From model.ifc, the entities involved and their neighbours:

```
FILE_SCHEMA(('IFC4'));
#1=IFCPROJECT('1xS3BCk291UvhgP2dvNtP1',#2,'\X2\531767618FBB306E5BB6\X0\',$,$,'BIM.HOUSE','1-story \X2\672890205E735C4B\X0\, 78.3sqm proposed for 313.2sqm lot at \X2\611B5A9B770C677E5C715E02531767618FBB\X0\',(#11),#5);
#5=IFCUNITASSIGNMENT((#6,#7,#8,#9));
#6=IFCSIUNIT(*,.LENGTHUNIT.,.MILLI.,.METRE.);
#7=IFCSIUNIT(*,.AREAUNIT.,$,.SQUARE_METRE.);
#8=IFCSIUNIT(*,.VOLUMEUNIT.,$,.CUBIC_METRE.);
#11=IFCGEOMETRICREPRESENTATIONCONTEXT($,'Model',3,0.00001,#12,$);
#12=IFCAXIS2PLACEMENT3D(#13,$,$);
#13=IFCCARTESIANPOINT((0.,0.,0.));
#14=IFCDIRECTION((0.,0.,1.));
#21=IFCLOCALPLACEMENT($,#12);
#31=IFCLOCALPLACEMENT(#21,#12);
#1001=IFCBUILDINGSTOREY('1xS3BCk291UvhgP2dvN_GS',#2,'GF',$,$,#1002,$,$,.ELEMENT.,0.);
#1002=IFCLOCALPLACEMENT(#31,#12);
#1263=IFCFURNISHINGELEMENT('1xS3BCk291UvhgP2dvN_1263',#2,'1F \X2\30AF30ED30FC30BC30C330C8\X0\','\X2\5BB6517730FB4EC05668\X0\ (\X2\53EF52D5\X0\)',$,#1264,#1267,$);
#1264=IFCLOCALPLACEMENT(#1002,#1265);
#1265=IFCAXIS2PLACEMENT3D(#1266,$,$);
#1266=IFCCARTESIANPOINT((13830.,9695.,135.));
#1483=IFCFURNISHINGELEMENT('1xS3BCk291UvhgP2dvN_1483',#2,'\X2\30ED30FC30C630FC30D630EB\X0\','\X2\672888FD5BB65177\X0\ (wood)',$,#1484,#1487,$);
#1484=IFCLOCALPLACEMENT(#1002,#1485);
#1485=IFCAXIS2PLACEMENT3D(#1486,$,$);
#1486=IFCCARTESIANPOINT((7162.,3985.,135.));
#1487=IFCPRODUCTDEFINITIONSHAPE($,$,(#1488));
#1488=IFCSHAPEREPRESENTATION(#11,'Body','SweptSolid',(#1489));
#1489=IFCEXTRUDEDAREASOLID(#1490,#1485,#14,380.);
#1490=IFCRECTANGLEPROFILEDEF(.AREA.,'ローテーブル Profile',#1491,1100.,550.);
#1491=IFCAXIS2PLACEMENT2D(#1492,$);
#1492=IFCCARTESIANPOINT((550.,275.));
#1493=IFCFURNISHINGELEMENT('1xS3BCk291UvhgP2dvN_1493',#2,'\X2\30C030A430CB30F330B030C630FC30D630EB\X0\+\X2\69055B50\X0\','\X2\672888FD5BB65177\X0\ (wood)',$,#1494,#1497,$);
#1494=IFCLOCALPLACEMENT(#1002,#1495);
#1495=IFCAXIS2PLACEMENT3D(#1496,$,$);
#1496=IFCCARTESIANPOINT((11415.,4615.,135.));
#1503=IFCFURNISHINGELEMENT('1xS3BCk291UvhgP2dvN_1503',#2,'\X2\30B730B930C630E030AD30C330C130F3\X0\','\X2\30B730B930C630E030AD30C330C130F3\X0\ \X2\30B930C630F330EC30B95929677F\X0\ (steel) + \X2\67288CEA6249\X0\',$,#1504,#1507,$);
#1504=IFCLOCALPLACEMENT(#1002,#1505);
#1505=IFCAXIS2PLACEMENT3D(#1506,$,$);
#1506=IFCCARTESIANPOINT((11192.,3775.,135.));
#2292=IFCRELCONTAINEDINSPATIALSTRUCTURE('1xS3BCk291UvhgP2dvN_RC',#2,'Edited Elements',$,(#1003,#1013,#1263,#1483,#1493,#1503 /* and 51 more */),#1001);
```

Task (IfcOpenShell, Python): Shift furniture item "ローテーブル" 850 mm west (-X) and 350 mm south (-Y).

```python
import ifcopenshell
import ifcopenshell.api.geometry
import ifcopenshell.util.placement

model = ifcopenshell.open("model.ifc")

item = model.by_guid("1xS3BCk291UvhgP2dvN_1483")
matrix = ifcopenshell.util.placement.get_local_placement(item.ObjectPlacement)
matrix[0, 3] -= 850.0
matrix[1, 3] -= 350.0
ifcopenshell.api.geometry.edit_object_placement(model, product=item, matrix=matrix, is_si=False)

print(ifcopenshell.util.placement.get_local_placement(item.ObjectPlacement).round(3) + 0.0)

model.write("model-out.ifc")
```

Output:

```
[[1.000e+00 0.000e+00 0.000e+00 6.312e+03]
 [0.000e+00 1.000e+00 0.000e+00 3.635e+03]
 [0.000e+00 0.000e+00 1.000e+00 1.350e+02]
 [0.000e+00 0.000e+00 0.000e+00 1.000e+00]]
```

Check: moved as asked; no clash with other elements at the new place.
